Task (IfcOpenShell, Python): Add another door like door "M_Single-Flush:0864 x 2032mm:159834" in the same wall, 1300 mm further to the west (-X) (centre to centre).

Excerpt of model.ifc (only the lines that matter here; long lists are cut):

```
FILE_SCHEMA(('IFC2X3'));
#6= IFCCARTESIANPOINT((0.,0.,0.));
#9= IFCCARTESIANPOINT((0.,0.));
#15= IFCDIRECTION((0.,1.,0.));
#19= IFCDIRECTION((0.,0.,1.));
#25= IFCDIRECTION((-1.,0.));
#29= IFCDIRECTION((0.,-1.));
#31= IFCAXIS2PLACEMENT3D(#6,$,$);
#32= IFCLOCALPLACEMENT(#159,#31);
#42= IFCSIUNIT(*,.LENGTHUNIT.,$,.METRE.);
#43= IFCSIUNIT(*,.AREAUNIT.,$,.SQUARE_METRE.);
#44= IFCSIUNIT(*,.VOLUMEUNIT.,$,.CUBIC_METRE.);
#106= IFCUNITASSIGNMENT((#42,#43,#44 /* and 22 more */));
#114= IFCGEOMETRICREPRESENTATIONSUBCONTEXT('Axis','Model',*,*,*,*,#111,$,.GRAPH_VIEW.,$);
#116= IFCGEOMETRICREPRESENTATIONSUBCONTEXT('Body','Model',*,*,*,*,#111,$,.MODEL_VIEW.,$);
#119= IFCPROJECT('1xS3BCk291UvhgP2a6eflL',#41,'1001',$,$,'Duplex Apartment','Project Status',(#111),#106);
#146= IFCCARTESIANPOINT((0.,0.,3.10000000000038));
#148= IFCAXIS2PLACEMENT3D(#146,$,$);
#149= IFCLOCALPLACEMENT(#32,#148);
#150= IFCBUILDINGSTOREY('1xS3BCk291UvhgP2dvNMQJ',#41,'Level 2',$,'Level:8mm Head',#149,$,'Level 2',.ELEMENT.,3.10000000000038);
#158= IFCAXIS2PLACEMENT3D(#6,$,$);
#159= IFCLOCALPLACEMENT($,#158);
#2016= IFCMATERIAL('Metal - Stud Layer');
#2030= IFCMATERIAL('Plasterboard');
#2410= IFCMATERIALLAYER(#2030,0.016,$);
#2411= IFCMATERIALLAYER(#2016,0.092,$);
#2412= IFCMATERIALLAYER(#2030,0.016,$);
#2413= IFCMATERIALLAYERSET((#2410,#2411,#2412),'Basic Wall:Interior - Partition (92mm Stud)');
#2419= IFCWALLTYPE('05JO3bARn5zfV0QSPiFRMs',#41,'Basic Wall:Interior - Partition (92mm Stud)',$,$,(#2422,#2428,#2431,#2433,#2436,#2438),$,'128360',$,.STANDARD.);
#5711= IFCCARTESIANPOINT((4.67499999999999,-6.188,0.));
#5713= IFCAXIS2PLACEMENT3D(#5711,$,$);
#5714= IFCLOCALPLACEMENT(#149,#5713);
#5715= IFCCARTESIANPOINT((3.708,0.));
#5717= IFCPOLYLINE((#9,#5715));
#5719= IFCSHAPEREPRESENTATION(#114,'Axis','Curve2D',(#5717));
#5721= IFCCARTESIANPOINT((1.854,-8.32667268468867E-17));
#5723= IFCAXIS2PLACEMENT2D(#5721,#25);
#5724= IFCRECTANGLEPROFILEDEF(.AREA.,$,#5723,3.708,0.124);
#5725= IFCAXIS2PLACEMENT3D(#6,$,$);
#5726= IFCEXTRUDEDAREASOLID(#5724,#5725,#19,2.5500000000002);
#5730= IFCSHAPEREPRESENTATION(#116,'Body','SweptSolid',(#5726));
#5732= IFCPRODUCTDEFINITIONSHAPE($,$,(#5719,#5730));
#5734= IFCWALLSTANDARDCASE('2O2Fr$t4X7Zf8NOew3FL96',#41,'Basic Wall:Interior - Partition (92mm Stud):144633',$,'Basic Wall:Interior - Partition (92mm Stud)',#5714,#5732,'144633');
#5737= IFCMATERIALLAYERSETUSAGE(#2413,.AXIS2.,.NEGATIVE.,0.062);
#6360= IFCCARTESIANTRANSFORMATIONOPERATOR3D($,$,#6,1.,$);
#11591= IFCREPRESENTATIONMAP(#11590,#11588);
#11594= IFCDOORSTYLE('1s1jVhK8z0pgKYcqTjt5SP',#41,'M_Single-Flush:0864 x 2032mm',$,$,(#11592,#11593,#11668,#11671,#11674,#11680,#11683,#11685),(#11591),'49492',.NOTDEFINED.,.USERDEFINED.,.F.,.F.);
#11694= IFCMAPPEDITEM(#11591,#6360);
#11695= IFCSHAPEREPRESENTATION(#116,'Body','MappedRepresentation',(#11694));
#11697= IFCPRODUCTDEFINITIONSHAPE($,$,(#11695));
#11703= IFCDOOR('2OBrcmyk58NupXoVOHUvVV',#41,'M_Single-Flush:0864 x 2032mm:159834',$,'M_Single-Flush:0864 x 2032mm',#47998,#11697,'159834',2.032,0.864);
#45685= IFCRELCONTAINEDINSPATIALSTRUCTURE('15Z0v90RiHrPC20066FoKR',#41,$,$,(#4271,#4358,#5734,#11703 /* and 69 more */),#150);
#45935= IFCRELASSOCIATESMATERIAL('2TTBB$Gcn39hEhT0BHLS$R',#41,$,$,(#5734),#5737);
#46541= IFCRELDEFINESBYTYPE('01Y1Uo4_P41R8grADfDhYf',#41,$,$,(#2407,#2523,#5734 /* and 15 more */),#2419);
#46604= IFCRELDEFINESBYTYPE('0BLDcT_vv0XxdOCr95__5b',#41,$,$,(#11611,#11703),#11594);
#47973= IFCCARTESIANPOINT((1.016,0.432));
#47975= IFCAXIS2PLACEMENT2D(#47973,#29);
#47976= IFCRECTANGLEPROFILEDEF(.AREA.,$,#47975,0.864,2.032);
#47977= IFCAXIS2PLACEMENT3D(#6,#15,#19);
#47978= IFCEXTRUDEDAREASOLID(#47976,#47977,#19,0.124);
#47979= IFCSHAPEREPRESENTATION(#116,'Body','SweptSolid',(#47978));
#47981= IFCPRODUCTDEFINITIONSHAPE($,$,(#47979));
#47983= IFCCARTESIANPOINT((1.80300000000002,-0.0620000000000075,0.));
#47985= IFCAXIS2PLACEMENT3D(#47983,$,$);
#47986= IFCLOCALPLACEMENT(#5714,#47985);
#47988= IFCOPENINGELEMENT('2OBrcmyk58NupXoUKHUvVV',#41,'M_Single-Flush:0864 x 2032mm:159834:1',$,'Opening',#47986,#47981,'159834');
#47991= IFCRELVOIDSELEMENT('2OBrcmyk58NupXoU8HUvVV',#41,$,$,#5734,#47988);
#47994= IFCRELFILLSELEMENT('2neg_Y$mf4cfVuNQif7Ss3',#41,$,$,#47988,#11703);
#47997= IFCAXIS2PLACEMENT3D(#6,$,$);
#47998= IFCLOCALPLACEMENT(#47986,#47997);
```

```python
import ifcopenshell
import ifcopenshell.api.feature
import ifcopenshell.api.geometry
import ifcopenshell.api.root
import ifcopenshell.geom
import ifcopenshell.util.element
import ifcopenshell.util.placement
import ifcopenshell.util.shape

model = ifcopenshell.open("model.ifc")
settings = ifcopenshell.geom.settings()


def volume(element):
    """Net volume in cubic metres, openings subtracted."""
    shape = ifcopenshell.geom.create_shape(settings, element)
    return ifcopenshell.util.shape.get_volume(shape.geometry)


def reuse_history(source, copy):
    """copy_class also copies each property set's owner history, people and application; keep the originals."""
    for rel in copy.IsDefinedBy:
        if rel.is_a("IfcRelDefinesByProperties") and (history := rel.RelatingPropertyDefinition.OwnerHistory):
            rel.RelatingPropertyDefinition.OwnerHistory = source.OwnerHistory
            ifcopenshell.util.element.remove_deep2(model, history)


door = model.by_guid("2OBrcmyk58NupXoVOHUvVV")
opening = door.FillsVoids[0].RelatingOpeningElement
wall = opening.VoidsElements[0].RelatingBuildingElement
before = volume(wall)
shift = ifcopenshell.util.placement.get_local_placement(wall.ObjectPlacement)[:3, 0] * -1.3

# copy_class copies the void relationship, type, container and properties, but no geometry.
new_opening = ifcopenshell.api.root.copy_class(model, product=opening)
new_opening.Representation = ifcopenshell.util.element.copy_deep(
    model, opening.Representation, exclude=["IfcGeometricRepresentationContext", "IfcRepresentationMap"]
)
new_opening.Name = "M_Single-Flush:0864 x 2032mm"
new_opening.Tag = None
new_door = ifcopenshell.api.root.copy_class(model, product=door)
new_door.Representation = ifcopenshell.util.element.copy_deep(
    model, door.Representation, exclude=["IfcGeometricRepresentationContext", "IfcRepresentationMap"]
)
new_door.Name = "M_Single-Flush:0864 x 2032mm"
new_door.Tag = None
reuse_history(door, new_door)
fills = ifcopenshell.api.feature.add_filling(model, opening=new_opening, element=new_door)
fills.OwnerHistory = new_door.OwnerHistory  # required in IFC2X3

for old, new in ((opening, new_opening), (door, new_door)):
    matrix = ifcopenshell.util.placement.get_local_placement(old.ObjectPlacement)
    matrix[:3, 3] += shift
    ifcopenshell.api.geometry.edit_object_placement(model, product=new, matrix=matrix, is_si=False)

after = volume(wall)

print(f"wall volume {before:.3f} -> {after:.3f} m3")

model.write("model_edited.ifc")
```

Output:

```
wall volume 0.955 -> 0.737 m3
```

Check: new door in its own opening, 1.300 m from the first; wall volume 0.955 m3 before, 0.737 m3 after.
